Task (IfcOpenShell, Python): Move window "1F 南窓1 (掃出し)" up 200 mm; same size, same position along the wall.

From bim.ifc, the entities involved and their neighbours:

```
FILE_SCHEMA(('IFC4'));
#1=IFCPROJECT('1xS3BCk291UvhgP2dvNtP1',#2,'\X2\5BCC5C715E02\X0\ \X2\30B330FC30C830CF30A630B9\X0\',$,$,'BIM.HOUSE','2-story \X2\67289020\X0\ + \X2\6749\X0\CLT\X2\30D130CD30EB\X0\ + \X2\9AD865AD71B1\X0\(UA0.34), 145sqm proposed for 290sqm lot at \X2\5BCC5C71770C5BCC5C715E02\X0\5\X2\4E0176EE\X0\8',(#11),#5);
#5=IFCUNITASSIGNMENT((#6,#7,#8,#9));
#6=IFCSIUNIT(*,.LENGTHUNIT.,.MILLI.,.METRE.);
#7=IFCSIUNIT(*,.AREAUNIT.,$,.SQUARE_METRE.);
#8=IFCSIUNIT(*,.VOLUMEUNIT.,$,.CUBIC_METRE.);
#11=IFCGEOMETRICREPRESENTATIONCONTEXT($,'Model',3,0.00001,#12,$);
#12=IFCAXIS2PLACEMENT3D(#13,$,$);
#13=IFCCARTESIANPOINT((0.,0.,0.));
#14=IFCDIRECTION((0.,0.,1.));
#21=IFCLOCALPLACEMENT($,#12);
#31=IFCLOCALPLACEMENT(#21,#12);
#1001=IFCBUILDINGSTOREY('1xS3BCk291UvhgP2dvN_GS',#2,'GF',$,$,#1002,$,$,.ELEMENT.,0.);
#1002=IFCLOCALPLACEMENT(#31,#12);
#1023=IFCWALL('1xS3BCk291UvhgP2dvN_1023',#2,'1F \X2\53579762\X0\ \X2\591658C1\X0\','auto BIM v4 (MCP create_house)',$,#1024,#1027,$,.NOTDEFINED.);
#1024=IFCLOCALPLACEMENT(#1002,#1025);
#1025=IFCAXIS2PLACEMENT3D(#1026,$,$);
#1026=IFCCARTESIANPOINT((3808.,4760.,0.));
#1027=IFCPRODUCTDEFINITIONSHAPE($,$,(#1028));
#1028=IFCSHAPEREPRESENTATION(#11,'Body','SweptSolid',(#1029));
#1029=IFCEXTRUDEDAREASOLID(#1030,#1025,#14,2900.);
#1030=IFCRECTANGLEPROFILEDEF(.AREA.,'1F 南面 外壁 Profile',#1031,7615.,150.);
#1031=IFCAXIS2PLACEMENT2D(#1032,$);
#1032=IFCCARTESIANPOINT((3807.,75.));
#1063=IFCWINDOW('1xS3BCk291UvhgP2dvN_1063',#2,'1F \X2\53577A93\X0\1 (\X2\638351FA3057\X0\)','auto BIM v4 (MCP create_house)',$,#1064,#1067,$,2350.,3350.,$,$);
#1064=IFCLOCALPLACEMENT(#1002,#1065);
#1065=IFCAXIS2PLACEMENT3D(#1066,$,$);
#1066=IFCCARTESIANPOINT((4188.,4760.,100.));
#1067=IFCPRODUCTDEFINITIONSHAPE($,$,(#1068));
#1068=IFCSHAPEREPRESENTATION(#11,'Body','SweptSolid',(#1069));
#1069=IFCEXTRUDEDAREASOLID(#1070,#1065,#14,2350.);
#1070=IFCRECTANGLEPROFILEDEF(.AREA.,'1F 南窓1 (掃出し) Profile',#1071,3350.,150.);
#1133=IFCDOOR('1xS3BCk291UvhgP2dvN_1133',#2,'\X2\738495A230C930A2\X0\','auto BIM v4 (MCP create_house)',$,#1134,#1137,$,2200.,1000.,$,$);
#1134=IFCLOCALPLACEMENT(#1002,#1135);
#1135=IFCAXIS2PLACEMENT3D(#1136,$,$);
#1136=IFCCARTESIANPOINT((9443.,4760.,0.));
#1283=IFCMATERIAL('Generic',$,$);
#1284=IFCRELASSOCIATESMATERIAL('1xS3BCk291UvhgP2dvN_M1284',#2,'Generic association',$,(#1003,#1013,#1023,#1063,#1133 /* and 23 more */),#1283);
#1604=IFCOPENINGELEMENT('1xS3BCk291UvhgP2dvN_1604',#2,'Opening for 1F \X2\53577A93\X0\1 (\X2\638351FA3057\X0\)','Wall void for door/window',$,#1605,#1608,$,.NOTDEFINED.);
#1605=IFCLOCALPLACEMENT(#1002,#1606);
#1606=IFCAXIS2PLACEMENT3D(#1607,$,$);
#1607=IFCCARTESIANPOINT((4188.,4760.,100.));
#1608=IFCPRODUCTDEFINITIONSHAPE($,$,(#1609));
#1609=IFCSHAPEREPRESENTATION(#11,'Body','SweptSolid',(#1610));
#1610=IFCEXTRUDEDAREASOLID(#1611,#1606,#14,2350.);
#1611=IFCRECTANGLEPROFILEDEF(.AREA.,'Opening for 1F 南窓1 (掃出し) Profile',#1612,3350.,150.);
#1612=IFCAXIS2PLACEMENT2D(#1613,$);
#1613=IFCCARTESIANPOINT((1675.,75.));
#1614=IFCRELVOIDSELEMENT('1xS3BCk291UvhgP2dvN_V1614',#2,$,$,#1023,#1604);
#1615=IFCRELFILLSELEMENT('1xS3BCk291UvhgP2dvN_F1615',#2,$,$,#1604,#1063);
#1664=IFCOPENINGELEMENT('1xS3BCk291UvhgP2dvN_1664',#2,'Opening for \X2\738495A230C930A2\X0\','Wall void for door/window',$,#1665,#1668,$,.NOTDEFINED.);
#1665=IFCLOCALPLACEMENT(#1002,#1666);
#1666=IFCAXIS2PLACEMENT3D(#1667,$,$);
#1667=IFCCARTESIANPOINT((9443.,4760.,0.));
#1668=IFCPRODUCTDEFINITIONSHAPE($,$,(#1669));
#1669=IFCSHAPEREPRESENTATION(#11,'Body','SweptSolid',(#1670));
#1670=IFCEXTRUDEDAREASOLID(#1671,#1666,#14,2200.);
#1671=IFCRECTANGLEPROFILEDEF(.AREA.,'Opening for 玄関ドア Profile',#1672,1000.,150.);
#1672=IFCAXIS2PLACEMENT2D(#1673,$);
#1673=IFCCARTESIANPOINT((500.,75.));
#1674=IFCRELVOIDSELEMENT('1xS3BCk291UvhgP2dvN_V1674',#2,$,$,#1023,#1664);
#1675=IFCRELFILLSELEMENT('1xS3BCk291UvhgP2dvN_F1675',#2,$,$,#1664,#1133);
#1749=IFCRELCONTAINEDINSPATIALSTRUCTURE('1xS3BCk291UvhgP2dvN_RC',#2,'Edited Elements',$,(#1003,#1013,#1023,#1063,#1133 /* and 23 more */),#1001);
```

```python
import numpy as np
import ifcopenshell
import ifcopenshell.api.geometry
import ifcopenshell.util.placement
import ifcopenshell.util.unit

model = ifcopenshell.open("bim.ifc")
unit_scale = ifcopenshell.util.unit.calculate_unit_scale(model)

window = model.by_id(1063)
opening = window.FillsVoids[0].RelatingOpeningElement
dz = 0.2 / unit_scale

shift = np.array([0.0, 0.0, dz])
# The window is not placed relative to its opening, so move both.
for product in (opening, window):
    matrix = ifcopenshell.util.placement.get_local_placement(product.ObjectPlacement)
    matrix[:3, 3] += shift
    ifcopenshell.api.geometry.edit_object_placement(model, product=product, matrix=matrix, is_si=False)

print(f"moved by {dz * unit_scale:+.3f} m")

model.write("bim_rev.ifc")
```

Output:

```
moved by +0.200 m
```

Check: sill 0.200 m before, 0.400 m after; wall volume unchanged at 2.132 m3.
